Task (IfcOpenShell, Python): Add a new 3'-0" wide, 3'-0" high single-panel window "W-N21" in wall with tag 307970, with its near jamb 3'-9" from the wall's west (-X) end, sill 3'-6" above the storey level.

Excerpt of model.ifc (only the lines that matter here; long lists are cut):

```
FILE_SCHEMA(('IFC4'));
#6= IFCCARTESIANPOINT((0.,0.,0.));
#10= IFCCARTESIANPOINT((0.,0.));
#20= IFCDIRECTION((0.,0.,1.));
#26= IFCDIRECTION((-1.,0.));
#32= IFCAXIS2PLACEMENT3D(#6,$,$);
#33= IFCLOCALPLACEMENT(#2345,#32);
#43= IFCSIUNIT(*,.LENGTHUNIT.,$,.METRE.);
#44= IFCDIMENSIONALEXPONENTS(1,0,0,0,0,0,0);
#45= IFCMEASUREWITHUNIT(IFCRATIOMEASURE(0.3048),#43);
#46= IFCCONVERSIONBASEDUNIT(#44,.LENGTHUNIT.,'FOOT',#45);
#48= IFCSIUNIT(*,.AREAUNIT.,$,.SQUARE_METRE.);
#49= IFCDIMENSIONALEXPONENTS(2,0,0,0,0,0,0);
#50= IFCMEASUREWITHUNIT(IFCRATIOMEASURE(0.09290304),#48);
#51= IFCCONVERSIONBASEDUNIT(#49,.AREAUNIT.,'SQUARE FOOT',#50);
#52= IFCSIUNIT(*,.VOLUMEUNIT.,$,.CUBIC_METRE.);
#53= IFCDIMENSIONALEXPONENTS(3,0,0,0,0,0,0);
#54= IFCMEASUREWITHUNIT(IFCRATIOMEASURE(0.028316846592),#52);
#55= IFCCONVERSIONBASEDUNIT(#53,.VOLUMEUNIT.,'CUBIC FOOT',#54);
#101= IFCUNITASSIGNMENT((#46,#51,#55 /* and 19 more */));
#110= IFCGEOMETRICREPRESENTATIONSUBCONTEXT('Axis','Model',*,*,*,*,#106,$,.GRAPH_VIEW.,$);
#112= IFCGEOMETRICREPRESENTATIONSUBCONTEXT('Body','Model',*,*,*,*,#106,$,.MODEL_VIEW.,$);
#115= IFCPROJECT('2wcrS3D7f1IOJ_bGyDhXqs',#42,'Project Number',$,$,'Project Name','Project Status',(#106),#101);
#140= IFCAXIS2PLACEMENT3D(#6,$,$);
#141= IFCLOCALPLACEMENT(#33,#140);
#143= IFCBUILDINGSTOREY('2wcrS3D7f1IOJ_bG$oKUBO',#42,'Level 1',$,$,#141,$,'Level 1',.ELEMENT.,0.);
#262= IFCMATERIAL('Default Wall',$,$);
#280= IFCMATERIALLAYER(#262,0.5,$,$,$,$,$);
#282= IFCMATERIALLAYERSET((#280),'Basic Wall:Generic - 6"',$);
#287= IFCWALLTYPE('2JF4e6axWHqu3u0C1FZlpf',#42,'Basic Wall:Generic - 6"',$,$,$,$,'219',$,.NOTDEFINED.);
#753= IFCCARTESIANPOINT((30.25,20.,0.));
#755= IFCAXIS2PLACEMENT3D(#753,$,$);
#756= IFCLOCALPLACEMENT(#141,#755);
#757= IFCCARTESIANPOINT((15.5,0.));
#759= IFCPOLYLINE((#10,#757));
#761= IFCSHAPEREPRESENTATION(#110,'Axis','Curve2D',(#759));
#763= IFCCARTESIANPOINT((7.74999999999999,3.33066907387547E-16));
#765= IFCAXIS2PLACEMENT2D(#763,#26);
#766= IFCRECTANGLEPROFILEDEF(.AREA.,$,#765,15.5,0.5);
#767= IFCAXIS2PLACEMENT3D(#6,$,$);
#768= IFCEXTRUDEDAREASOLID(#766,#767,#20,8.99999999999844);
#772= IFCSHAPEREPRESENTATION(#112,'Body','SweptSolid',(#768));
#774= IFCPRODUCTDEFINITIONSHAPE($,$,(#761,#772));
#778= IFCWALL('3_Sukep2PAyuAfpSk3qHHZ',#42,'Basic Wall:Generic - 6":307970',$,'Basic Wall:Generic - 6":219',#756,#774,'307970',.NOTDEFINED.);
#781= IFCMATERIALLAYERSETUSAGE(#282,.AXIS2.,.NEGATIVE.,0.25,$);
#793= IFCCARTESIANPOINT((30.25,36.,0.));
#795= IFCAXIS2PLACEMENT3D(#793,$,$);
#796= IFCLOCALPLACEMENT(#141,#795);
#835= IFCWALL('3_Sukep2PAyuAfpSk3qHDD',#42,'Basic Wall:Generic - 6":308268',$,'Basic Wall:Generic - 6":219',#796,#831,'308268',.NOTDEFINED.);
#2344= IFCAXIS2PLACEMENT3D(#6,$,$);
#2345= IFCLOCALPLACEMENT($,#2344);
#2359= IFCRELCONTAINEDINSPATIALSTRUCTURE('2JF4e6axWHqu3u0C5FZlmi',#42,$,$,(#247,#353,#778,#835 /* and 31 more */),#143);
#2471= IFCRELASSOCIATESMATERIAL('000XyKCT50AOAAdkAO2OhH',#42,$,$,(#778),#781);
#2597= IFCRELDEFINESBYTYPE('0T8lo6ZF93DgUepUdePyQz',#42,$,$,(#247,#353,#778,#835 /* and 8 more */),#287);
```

```python
import numpy as np
import ifcopenshell
import ifcopenshell.api.feature
import ifcopenshell.api.geometry
import ifcopenshell.api.root
import ifcopenshell.api.spatial
import ifcopenshell.geom
import ifcopenshell.util.element
import ifcopenshell.util.placement
import ifcopenshell.util.representation
import ifcopenshell.util.shape
import ifcopenshell.util.unit

model = ifcopenshell.open("model.ifc")
unit_scale = ifcopenshell.util.unit.calculate_unit_scale(model)
settings = ifcopenshell.geom.settings()


def volume(element):
    """Net volume in cubic metres, openings subtracted."""
    shape = ifcopenshell.geom.create_shape(settings, element)
    return ifcopenshell.util.shape.get_volume(shape.geometry)


wall = model.by_guid("3_Sukep2PAyuAfpSk3qHHZ")
storey = ifcopenshell.util.element.get_container(wall, ifc_class="IfcBuildingStorey")
context = ifcopenshell.util.representation.get_context(model, "Model", "Body", "MODEL_VIEW")
before = volume(wall)

width, height, from_end, sill = 0.9144, 0.9144, 1.143, 1.0668  # metres

# The wall runs along its own X axis, and the end named is its -X end.
wall_shape = ifcopenshell.geom.create_shape(settings, wall)
x, y, z = ifcopenshell.util.shape.get_vertices(wall_shape.geometry).T
start = x.min() + from_end
face, thickness = float(y.min()), float(y.max() - y.min())
wall_matrix = ifcopenshell.util.placement.get_local_placement(wall.ObjectPlacement)
level = ifcopenshell.util.placement.get_local_placement(storey.ObjectPlacement)[2, 3]


def in_wall(x, y):
    """Placement at x, y metres in the wall's axes, at sill height."""
    matrix = wall_matrix.copy()
    matrix[:, 3] = wall_matrix @ np.array([x / unit_scale, y / unit_scale, 0.0, 1.0])
    matrix[2, 3] = level + sill / unit_scale
    return matrix


# Opening: a box that overshoots both wall faces by 50 mm.
opening = ifcopenshell.api.root.create_entity(model, ifc_class="IfcOpeningElement", predefined_type="OPENING")
box = ifcopenshell.api.geometry.add_wall_representation(
    model, context=context, length=width, height=height, thickness=thickness + 0.1
)
ifcopenshell.api.geometry.assign_representation(model, product=opening, representation=box)
ifcopenshell.api.geometry.edit_object_placement(model, product=opening, matrix=in_wall(start, face - 0.05), is_si=False)
ifcopenshell.api.feature.add_feature(model, feature=opening, element=wall)

window = ifcopenshell.api.root.create_entity(model, ifc_class="IfcWindow", name="W-N21", predefined_type="WINDOW")
window.OverallWidth, window.OverallHeight = width / unit_scale, height / unit_scale
window.PartitioningType = "SINGLE_PANEL"
body = ifcopenshell.api.geometry.add_window_representation(
    model,
    context=context,
    overall_width=window.OverallWidth,
    overall_height=window.OverallHeight,
    partition_type="SINGLE_PANEL",
)
ifcopenshell.api.geometry.assign_representation(model, product=window, representation=body)
ifcopenshell.api.spatial.assign_container(model, products=[window], relating_structure=storey)
ifcopenshell.api.feature.add_filling(model, opening=opening, element=window)

# Centre the window in the wall's thickness.
ifcopenshell.api.geometry.edit_object_placement(model, product=window, matrix=in_wall(start, face), is_si=False)
window_shape = ifcopenshell.geom.create_shape(settings, window)
depth = ifcopenshell.util.shape.get_vertices(window_shape.geometry)[:, 1]
offset = face + thickness / 2 - (depth.min() + depth.max()) / 2
ifcopenshell.api.geometry.edit_object_placement(model, product=window, matrix=in_wall(start, offset), is_si=False)

after = volume(wall)

print(f"wall volume {before:.3f} -> {after:.3f} m3")

model.write("model-out.ifc")
```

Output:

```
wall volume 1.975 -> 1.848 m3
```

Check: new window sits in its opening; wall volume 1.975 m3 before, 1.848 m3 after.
